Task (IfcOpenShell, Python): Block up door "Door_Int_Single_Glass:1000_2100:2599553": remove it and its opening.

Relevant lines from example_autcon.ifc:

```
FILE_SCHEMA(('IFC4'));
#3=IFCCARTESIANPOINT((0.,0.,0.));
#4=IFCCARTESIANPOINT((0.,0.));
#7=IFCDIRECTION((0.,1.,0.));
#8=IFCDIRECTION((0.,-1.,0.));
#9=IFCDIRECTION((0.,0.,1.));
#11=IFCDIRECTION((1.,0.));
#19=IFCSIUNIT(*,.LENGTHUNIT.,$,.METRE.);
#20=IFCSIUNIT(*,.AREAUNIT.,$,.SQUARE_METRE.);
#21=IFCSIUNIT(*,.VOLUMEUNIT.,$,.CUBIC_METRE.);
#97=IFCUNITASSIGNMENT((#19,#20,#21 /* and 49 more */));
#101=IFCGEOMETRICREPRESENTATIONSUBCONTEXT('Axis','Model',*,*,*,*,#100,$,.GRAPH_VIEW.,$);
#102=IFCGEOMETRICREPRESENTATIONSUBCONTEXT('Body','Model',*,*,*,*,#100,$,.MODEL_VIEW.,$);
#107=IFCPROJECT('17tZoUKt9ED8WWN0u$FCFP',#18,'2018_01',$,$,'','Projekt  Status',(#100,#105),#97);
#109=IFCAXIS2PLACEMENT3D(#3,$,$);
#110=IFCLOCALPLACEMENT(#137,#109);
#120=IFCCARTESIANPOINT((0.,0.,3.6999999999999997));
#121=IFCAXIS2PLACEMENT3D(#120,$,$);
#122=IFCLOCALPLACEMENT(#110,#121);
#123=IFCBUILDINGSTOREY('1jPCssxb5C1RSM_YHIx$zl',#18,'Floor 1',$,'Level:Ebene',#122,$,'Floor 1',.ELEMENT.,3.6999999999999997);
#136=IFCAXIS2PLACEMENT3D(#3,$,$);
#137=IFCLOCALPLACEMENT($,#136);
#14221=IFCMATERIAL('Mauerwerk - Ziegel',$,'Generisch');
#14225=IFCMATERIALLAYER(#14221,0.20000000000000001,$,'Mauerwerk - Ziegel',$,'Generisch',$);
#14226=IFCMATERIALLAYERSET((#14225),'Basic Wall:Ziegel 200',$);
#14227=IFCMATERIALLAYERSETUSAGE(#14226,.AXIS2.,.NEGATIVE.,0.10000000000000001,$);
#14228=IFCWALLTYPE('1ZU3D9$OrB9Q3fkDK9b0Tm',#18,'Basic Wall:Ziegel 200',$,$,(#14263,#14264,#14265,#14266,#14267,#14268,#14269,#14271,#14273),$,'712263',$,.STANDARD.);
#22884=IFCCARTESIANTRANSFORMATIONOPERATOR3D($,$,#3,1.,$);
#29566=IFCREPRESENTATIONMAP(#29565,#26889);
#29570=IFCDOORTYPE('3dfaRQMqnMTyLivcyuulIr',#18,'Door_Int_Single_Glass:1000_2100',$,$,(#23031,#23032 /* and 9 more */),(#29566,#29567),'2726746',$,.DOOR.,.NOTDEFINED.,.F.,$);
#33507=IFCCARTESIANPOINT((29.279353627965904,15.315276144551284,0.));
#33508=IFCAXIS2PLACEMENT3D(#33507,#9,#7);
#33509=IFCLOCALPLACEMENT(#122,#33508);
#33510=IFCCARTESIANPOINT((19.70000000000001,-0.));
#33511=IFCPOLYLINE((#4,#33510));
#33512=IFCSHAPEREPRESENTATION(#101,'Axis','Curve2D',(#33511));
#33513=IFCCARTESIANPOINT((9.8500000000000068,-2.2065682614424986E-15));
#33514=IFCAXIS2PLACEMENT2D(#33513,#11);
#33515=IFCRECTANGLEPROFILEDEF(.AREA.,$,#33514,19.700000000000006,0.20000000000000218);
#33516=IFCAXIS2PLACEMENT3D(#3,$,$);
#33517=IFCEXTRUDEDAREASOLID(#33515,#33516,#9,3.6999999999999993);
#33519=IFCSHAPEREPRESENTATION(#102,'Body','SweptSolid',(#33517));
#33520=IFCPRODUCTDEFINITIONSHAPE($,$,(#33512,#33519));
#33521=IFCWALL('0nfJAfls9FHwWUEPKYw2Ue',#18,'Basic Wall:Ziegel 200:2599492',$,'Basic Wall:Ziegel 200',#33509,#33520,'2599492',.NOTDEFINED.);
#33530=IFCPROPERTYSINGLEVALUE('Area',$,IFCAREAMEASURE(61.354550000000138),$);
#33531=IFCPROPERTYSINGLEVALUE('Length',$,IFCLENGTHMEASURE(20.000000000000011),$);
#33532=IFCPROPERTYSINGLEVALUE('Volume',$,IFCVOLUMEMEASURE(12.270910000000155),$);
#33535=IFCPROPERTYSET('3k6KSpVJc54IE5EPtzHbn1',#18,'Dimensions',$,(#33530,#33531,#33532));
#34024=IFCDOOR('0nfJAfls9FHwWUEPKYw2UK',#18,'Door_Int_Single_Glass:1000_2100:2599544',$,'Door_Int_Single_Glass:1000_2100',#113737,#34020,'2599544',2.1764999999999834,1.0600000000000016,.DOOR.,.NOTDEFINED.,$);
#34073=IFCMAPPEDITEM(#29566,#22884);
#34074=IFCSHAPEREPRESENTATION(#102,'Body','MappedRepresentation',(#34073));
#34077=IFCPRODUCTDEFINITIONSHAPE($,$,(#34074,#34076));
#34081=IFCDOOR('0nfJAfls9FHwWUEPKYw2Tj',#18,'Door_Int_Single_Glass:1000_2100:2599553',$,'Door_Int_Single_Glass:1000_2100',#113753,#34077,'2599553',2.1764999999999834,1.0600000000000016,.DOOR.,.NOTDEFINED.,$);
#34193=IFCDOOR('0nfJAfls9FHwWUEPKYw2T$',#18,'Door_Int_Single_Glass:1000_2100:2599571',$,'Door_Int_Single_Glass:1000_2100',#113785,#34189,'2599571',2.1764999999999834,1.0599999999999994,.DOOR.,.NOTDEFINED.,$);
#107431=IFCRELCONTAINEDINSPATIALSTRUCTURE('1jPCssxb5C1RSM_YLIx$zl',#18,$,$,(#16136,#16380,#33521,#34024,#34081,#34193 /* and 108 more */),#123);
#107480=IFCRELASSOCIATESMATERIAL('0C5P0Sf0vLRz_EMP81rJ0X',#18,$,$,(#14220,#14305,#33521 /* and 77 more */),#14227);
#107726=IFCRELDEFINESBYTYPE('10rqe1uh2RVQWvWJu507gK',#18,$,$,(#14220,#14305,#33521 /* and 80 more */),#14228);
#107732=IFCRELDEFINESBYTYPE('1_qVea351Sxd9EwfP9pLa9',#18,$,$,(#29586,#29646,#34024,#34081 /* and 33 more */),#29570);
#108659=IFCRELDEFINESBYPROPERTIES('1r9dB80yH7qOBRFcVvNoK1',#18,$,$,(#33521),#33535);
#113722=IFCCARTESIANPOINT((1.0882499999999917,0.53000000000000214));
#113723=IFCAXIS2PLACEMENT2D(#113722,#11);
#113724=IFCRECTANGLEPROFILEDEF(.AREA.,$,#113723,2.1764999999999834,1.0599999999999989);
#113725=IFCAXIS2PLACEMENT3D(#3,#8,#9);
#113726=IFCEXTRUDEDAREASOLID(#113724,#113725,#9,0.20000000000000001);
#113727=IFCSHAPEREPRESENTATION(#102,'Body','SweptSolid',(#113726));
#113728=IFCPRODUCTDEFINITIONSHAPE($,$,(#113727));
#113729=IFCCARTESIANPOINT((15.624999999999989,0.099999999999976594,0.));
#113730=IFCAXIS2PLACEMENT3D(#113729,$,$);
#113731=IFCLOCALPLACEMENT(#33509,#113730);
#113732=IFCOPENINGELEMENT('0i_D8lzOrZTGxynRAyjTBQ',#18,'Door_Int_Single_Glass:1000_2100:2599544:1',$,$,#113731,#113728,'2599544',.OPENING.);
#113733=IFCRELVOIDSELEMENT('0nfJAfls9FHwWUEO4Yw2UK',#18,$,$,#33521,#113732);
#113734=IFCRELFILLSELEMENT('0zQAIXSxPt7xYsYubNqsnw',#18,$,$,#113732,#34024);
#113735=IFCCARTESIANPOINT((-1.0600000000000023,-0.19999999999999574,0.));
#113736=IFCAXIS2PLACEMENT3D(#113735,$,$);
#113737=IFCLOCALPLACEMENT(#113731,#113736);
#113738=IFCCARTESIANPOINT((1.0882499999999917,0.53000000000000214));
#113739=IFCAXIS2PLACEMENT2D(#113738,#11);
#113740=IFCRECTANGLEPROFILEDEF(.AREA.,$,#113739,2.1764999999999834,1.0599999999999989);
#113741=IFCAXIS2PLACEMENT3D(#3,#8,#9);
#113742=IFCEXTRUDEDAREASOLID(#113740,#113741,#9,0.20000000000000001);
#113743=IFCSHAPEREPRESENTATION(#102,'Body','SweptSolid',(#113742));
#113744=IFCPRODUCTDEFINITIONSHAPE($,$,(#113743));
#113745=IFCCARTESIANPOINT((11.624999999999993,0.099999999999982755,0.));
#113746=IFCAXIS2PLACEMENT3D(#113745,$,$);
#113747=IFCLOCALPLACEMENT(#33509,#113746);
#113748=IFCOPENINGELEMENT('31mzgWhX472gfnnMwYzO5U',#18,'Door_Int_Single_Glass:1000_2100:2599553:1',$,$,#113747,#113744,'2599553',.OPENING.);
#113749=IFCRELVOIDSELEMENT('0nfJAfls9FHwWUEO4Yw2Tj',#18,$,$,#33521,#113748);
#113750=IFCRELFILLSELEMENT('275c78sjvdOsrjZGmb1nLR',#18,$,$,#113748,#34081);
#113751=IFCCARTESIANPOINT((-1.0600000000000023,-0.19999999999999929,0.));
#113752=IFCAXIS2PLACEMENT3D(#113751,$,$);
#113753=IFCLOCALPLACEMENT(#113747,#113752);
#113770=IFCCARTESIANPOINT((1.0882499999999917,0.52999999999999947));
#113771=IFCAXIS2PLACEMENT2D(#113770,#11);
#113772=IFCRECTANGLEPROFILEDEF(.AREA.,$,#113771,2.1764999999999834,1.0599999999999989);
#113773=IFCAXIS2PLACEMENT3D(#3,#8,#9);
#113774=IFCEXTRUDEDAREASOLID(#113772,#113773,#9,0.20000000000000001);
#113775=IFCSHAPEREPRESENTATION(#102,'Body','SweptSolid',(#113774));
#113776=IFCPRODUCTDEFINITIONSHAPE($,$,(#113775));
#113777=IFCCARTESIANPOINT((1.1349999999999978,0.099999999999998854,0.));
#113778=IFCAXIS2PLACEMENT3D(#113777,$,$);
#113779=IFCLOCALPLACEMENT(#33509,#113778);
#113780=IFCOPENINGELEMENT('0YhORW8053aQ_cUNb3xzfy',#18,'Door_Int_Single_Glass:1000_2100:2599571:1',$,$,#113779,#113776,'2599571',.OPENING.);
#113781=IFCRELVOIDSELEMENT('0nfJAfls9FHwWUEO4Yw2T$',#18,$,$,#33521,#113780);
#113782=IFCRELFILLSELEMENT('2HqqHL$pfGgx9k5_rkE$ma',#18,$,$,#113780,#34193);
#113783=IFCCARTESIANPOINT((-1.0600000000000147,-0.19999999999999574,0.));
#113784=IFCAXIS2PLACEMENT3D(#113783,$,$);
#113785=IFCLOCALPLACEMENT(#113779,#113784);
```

```python
import ifcopenshell
import ifcopenshell.api.feature
import ifcopenshell.api.pset
import ifcopenshell.api.root
import ifcopenshell.geom
import ifcopenshell.util.element
import ifcopenshell.util.shape
import ifcopenshell.util.unit

model = ifcopenshell.open("example_autcon.ifc")
area_scale = ifcopenshell.util.unit.calculate_unit_scale(model, "AREAUNIT")
volume_scale = ifcopenshell.util.unit.calculate_unit_scale(model, "VOLUMEUNIT")
settings = ifcopenshell.geom.settings()


def volume(element):
    """Net volume in cubic metres, openings subtracted."""
    shape = ifcopenshell.geom.create_shape(settings, element)
    return ifcopenshell.util.shape.get_volume(shape.geometry)


door = model.by_guid("0nfJAfls9FHwWUEPKYw2Tj")
opening = door.FillsVoids[0].RelatingOpeningElement
wall = opening.VoidsElements[0].RelatingBuildingElement
before = volume(wall)

ifcopenshell.api.root.remove_product(model, product=door)
ifcopenshell.api.feature.remove_feature(model, feature=opening)

after = volume(wall)
thickness = 0.2  # wall thickness in metres

# Update the wall's stored quantities.
pset = model.by_id(ifcopenshell.util.element.get_pset(wall, "Dimensions", should_inherit=False)["id"])
ifcopenshell.api.pset.edit_pset(model, pset=pset, properties={
    "Area": model.create_entity("IfcAreaMeasure", after / thickness / area_scale),
    "Volume": model.create_entity("IfcVolumeMeasure", after / volume_scale),
})

print(f"wall volume {before:.3f} -> {after:.3f} m3")

model.write("example_autcon-out.ifc")
```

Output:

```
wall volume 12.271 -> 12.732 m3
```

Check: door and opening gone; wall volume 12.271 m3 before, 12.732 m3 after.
